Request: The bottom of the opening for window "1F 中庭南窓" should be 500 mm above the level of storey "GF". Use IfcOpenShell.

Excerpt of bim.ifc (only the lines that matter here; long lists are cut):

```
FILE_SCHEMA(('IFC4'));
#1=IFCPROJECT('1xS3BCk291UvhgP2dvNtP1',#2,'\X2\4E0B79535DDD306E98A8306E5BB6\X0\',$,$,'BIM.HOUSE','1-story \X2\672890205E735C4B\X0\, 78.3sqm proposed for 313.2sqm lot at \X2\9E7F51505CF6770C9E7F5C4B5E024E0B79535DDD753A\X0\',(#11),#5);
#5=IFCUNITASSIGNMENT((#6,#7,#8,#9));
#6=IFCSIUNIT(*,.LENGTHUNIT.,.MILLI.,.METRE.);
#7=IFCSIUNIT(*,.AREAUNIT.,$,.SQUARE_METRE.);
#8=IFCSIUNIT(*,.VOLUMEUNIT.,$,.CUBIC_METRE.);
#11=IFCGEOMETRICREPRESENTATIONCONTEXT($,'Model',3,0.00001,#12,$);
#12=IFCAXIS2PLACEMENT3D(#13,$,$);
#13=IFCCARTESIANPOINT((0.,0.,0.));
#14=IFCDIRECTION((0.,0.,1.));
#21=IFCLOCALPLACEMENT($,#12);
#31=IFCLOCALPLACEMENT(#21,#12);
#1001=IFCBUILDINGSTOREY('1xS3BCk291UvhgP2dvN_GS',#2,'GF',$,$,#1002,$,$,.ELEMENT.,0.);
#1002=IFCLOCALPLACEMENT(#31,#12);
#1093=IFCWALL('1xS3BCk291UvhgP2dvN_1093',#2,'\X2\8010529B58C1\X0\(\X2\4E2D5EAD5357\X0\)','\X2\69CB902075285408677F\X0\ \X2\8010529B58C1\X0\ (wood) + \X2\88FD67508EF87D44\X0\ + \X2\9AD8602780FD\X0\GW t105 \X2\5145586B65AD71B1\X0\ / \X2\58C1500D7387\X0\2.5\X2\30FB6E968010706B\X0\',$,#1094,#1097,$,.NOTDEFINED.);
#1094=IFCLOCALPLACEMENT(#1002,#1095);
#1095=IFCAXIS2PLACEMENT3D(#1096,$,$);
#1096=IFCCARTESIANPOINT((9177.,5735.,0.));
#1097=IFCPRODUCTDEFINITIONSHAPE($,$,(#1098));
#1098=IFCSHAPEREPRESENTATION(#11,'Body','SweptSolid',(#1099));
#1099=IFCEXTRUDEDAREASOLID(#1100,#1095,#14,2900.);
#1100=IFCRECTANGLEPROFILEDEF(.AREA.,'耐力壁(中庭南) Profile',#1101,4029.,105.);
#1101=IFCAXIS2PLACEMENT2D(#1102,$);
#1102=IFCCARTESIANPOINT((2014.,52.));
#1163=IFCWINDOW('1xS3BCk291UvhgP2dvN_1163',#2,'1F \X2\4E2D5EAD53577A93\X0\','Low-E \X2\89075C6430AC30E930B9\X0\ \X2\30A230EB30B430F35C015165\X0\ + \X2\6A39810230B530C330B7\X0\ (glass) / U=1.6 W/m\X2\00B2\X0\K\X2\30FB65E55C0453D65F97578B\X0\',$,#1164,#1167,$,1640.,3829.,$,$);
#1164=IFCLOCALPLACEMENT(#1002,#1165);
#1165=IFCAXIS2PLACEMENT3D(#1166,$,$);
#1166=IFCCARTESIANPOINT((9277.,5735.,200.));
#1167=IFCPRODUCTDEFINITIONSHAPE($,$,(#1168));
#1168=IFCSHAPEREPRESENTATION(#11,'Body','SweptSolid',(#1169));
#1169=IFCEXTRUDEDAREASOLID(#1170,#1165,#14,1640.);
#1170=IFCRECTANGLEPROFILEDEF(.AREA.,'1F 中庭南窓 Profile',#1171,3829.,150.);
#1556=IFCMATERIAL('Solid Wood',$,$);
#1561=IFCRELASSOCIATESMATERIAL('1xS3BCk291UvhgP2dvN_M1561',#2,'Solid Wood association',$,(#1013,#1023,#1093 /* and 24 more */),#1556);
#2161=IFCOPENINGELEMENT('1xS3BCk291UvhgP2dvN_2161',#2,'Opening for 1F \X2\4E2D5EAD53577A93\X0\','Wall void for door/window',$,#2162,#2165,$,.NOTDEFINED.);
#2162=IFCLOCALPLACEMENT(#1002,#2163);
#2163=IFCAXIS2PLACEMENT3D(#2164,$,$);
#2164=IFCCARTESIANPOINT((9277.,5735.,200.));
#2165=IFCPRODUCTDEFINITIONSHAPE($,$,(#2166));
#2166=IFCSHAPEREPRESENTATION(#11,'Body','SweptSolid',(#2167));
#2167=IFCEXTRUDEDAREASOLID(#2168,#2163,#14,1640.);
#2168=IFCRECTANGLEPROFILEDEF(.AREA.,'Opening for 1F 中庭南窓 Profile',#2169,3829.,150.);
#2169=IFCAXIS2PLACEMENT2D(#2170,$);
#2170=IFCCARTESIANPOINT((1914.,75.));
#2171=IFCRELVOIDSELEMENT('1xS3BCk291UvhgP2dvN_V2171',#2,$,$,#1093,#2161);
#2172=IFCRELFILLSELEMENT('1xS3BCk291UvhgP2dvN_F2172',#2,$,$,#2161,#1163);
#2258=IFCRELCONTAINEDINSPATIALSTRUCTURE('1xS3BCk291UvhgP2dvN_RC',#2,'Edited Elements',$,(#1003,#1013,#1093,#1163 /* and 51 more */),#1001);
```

```python
import numpy as np
import ifcopenshell
import ifcopenshell.api.geometry
import ifcopenshell.geom
import ifcopenshell.util.element
import ifcopenshell.util.placement
import ifcopenshell.util.shape
import ifcopenshell.util.unit

model = ifcopenshell.open("bim.ifc")
unit_scale = ifcopenshell.util.unit.calculate_unit_scale(model)

window = model.by_guid("1xS3BCk291UvhgP2dvN_1163")
opening = window.FillsVoids[0].RelatingOpeningElement
storey = ifcopenshell.util.element.get_container(window, ifc_class="IfcBuildingStorey")
level = ifcopenshell.util.placement.get_local_placement(storey.ObjectPlacement)[2, 3]

# The opening's origin need not be at the sill, so measure its lowest point.
shape = ifcopenshell.geom.create_shape(ifcopenshell.geom.settings(), opening)
bottom = ifcopenshell.util.shape.get_shape_bottom_elevation(shape, shape.geometry) / unit_scale
dz = level + 500.0 - bottom

shift = np.array([0.0, 0.0, dz])
# The window is not placed relative to its opening, so move both.
for product in (opening, window):
    matrix = ifcopenshell.util.placement.get_local_placement(product.ObjectPlacement)
    matrix[:3, 3] += shift
    ifcopenshell.api.geometry.edit_object_placement(model, product=product, matrix=matrix, is_si=False)

print(f"moved by {dz * unit_scale:+.3f} m")

model.write("bim_edited.ifc")
```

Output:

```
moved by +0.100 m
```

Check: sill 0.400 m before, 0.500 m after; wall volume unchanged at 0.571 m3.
